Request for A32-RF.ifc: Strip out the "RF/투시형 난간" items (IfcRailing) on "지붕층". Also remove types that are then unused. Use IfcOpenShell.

First a look at what the model holds.

```python
import ifcopenshell
import ifcopenshell.util.element

model = ifcopenshell.open("A32-RF.ifc")
print(model.schema)
storey = next(s for s in model.by_type("IfcBuildingStorey") if s.Name == "지붕층")
railings = [e for e in ifcopenshell.util.element.get_decomposition(storey) if e.is_a("IfcRailing")]
seen = {}
for e in railings:
    element_type = ifcopenshell.util.element.get_type(e)
    name = element_type.Name if element_type not in (None, e) else None
    seen[name] = seen.get(name, 0) + 1
for name, count in sorted(seen.items(), key=str):
    print(count, "x", name)
```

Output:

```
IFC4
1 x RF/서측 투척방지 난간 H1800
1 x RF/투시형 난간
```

```python
import ifcopenshell
import ifcopenshell.api.root
import ifcopenshell.util.element

model = ifcopenshell.open("A32-RF.ifc")

storey = next(s for s in model.by_type("IfcBuildingStorey") if s.Name == "지붕층")
railings = [e for e in ifcopenshell.util.element.get_decomposition(storey) if e.is_a("IfcRailing")]
targets = [e for e in railings if (t := ifcopenshell.util.element.get_type(e)) not in (None, e) and t.Name == "RF/투시형 난간"]
types = {ifcopenshell.util.element.get_type(e) for e in targets} - {None, *targets}

for e in targets:
    ifcopenshell.api.root.remove_product(model, product=e)
print(len(targets), "removed")

unused = [t for t in types if not ifcopenshell.util.element.get_types(t)]
for t in unused:
    ifcopenshell.api.root.remove_product(model, product=t)
print(len(unused), "unused types removed")

model.write("A32-RF_updated.ifc")
```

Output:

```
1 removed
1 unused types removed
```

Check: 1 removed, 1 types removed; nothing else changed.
